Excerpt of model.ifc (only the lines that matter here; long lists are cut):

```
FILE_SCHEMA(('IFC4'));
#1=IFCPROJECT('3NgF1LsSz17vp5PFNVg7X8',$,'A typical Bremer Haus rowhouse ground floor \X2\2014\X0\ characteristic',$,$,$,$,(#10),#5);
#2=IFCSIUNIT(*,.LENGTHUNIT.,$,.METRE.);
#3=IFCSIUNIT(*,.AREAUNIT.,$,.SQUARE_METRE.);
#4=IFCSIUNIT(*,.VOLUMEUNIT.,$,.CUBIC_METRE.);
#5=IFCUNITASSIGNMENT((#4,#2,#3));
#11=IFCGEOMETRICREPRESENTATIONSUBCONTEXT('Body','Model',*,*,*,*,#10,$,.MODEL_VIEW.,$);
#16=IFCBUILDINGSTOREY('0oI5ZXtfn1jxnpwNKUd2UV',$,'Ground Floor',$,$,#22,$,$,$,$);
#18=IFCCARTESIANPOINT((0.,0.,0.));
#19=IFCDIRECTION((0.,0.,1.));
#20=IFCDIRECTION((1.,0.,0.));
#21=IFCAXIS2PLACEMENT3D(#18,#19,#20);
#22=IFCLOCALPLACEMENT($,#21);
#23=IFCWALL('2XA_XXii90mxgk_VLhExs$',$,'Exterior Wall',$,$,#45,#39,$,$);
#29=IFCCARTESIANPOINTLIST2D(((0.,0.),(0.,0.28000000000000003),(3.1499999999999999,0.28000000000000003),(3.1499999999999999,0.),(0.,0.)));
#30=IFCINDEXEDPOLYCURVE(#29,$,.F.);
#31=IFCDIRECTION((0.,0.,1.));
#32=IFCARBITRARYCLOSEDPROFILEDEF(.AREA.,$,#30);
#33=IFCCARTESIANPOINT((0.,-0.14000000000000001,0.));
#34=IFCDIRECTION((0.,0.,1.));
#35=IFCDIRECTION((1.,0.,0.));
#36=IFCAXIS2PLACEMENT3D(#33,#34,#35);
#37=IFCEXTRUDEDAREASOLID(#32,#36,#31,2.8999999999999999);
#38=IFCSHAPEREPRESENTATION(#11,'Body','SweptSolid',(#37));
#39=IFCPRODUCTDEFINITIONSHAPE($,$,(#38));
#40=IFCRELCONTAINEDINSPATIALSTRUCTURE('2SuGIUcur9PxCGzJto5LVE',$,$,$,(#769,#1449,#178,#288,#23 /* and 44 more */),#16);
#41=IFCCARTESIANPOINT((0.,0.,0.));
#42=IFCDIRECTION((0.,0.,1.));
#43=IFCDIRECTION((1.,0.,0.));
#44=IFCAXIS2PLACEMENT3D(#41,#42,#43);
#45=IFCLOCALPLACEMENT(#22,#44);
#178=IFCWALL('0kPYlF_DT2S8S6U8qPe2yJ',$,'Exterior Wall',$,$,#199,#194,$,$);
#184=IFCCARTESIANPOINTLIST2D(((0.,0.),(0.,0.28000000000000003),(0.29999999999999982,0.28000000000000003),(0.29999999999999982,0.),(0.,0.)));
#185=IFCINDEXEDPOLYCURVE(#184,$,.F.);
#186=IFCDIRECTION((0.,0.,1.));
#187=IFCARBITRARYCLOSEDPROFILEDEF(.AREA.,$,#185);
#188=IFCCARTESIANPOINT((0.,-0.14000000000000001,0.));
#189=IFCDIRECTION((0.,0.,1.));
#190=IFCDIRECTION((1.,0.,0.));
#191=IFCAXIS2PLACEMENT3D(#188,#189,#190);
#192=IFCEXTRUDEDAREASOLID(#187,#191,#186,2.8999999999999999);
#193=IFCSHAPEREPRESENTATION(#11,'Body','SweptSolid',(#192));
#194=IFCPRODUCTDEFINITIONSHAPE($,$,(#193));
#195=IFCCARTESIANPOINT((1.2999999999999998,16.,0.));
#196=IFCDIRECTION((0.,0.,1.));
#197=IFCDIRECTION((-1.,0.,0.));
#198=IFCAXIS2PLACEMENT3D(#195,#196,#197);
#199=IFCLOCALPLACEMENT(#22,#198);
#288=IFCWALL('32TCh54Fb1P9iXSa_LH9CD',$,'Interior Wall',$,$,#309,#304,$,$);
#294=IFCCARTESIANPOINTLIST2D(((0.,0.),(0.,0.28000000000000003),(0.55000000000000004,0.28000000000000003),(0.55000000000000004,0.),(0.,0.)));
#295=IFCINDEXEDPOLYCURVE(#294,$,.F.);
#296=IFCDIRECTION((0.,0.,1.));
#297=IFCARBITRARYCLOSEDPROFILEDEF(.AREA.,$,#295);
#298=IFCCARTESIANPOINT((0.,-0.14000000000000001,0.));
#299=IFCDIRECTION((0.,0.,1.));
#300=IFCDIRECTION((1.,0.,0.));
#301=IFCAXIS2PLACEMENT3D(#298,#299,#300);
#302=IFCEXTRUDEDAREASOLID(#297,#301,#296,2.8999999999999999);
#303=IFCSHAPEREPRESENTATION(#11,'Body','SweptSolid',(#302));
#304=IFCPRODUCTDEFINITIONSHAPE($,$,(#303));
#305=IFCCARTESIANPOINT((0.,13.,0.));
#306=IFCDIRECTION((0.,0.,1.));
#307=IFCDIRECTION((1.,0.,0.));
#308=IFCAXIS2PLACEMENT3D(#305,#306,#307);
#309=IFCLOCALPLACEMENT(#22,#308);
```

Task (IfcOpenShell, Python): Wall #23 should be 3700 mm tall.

```python
import ifcopenshell
import ifcopenshell.geom
import ifcopenshell.util.representation
import ifcopenshell.util.shape
import ifcopenshell.util.unit

model = ifcopenshell.open("model.ifc")
unit_scale = ifcopenshell.util.unit.calculate_unit_scale(model)
settings = ifcopenshell.geom.settings()


def volume(element):
    """Net volume in cubic metres, openings subtracted."""
    shape = ifcopenshell.geom.create_shape(settings, element)
    return ifcopenshell.util.shape.get_volume(shape.geometry)


wall = model.by_guid("2XA_XXii90mxgk_VLhExs$")
before = volume(wall)

body = ifcopenshell.util.representation.get_representation(wall, "Model", "Body")
solid = body.Items[0]
old_height = solid.Depth
solid.Depth = 3.7 / unit_scale
after = volume(wall)

print(f"height {old_height:g} -> {solid.Depth:g}, volume {before:.3f} -> {after:.3f} m3")

model.write("model_edited.ifc")
```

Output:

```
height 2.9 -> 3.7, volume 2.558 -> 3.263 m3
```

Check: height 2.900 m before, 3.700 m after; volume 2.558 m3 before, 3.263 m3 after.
